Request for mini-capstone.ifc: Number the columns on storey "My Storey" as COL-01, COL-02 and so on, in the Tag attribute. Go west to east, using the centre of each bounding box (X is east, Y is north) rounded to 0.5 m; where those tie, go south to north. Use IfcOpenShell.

First a look at what the model holds.

```python
import ifcopenshell
import ifcopenshell.util.element
import ifcopenshell.util.placement

model = ifcopenshell.open("mini-capstone.ifc")
print(model.schema)
storey = next(s for s in model.by_type("IfcBuildingStorey") if s.Name == "My Storey")
columns = [e for e in ifcopenshell.util.element.get_decomposition(storey) if e.is_a("IfcColumn")]
for e in sorted(columns, key=lambda e: e.id()):
    origin = ifcopenshell.util.placement.get_local_placement(e.ObjectPlacement)[:3, 3]
    print(e.id(), e.Tag, e.Name, origin.round(2) + 0.0, sep=" | ")
```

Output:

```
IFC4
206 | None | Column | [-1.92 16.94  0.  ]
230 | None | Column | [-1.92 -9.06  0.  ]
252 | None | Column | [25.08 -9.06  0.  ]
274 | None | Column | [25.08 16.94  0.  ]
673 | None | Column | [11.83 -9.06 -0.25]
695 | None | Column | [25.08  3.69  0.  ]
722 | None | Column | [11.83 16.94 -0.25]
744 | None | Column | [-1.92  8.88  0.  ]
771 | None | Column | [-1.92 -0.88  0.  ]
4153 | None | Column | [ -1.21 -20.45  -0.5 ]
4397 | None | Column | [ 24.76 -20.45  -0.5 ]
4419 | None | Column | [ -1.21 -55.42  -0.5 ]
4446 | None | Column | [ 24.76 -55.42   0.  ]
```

```python
import ifcopenshell
import ifcopenshell.geom
import ifcopenshell.util.element
import ifcopenshell.util.shape

model = ifcopenshell.open("mini-capstone.ifc")
settings = ifcopenshell.geom.settings()
settings.set("use-world-coords", True)


def centre(element):
    shape = ifcopenshell.geom.create_shape(settings, element)
    return ifcopenshell.util.shape.get_bbox_centroid(shape.geometry)


storey = next(s for s in model.by_type("IfcBuildingStorey") if s.Name == "My Storey")
columns = [e for e in ifcopenshell.util.element.get_decomposition(storey) if e.is_a("IfcColumn")]

# Insertion points can sit at a corner or the storey origin, so sort by the geometry (in metres).
centres = {e: centre(e) for e in columns}
columns.sort(key=lambda e: (round(centres[e][0] / 0.5), centres[e][1]))

for i, e in enumerate(columns, start=1):
    number = f"COL-{i:02d}"
    e.Tag = number
    print(e.id(), number)

model.write("mini-capstone_updated.ifc")
```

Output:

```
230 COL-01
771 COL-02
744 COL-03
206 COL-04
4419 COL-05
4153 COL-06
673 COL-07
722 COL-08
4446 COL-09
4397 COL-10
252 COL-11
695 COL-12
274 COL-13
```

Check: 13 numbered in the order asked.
